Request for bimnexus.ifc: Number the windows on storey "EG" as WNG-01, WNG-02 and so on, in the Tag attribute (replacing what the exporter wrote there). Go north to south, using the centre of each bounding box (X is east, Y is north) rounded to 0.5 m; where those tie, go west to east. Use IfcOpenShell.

First a look at what the model holds.

```python
import ifcopenshell
import ifcopenshell.util.element
import ifcopenshell.util.placement

model = ifcopenshell.open("bimnexus.ifc")
print(model.schema)
storey = next(s for s in model.by_type("IfcBuildingStorey") if s.Name == "EG")
windows = [e for e in ifcopenshell.util.element.get_decomposition(storey) if e.is_a("IfcWindow")]
for e in sorted(windows, key=lambda e: e.id()):
    origin = ifcopenshell.util.placement.get_local_placement(e.ObjectPlacement)[:3, 3]
    print(e.id(), e.Tag, e.Name, origin.round(2) + 0.0, sep=" | ")
```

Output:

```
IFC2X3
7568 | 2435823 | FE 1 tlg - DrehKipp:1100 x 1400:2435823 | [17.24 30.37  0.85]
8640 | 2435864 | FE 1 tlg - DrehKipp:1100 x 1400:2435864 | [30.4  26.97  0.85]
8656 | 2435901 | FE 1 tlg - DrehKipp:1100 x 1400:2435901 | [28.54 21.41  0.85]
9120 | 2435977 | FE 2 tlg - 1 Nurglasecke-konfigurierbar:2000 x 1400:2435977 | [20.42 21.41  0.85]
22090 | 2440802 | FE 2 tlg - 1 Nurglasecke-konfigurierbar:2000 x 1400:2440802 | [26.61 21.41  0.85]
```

```python
import ifcopenshell
import ifcopenshell.geom
import ifcopenshell.util.element
import ifcopenshell.util.shape

model = ifcopenshell.open("bimnexus.ifc")
settings = ifcopenshell.geom.settings()
settings.set("use-world-coords", True)


def centre(element):
    shape = ifcopenshell.geom.create_shape(settings, element)
    return ifcopenshell.util.shape.get_bbox_centroid(shape.geometry)


storey = next(s for s in model.by_type("IfcBuildingStorey") if s.Name == "EG")
windows = [e for e in ifcopenshell.util.element.get_decomposition(storey) if e.is_a("IfcWindow")]

# Insertion points can sit at a corner or the storey origin, so sort by the geometry (in metres).
centres = {e: centre(e) for e in windows}
windows.sort(key=lambda e: (-round(centres[e][1] / 0.5), centres[e][0]))

for i, e in enumerate(windows, start=1):
    number = f"WNG-{i:02d}"
    e.Tag = number
    print(e.id(), number)

model.write("bimnexus_updated.ifc")
```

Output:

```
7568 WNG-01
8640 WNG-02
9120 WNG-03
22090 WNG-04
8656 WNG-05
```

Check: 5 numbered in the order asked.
